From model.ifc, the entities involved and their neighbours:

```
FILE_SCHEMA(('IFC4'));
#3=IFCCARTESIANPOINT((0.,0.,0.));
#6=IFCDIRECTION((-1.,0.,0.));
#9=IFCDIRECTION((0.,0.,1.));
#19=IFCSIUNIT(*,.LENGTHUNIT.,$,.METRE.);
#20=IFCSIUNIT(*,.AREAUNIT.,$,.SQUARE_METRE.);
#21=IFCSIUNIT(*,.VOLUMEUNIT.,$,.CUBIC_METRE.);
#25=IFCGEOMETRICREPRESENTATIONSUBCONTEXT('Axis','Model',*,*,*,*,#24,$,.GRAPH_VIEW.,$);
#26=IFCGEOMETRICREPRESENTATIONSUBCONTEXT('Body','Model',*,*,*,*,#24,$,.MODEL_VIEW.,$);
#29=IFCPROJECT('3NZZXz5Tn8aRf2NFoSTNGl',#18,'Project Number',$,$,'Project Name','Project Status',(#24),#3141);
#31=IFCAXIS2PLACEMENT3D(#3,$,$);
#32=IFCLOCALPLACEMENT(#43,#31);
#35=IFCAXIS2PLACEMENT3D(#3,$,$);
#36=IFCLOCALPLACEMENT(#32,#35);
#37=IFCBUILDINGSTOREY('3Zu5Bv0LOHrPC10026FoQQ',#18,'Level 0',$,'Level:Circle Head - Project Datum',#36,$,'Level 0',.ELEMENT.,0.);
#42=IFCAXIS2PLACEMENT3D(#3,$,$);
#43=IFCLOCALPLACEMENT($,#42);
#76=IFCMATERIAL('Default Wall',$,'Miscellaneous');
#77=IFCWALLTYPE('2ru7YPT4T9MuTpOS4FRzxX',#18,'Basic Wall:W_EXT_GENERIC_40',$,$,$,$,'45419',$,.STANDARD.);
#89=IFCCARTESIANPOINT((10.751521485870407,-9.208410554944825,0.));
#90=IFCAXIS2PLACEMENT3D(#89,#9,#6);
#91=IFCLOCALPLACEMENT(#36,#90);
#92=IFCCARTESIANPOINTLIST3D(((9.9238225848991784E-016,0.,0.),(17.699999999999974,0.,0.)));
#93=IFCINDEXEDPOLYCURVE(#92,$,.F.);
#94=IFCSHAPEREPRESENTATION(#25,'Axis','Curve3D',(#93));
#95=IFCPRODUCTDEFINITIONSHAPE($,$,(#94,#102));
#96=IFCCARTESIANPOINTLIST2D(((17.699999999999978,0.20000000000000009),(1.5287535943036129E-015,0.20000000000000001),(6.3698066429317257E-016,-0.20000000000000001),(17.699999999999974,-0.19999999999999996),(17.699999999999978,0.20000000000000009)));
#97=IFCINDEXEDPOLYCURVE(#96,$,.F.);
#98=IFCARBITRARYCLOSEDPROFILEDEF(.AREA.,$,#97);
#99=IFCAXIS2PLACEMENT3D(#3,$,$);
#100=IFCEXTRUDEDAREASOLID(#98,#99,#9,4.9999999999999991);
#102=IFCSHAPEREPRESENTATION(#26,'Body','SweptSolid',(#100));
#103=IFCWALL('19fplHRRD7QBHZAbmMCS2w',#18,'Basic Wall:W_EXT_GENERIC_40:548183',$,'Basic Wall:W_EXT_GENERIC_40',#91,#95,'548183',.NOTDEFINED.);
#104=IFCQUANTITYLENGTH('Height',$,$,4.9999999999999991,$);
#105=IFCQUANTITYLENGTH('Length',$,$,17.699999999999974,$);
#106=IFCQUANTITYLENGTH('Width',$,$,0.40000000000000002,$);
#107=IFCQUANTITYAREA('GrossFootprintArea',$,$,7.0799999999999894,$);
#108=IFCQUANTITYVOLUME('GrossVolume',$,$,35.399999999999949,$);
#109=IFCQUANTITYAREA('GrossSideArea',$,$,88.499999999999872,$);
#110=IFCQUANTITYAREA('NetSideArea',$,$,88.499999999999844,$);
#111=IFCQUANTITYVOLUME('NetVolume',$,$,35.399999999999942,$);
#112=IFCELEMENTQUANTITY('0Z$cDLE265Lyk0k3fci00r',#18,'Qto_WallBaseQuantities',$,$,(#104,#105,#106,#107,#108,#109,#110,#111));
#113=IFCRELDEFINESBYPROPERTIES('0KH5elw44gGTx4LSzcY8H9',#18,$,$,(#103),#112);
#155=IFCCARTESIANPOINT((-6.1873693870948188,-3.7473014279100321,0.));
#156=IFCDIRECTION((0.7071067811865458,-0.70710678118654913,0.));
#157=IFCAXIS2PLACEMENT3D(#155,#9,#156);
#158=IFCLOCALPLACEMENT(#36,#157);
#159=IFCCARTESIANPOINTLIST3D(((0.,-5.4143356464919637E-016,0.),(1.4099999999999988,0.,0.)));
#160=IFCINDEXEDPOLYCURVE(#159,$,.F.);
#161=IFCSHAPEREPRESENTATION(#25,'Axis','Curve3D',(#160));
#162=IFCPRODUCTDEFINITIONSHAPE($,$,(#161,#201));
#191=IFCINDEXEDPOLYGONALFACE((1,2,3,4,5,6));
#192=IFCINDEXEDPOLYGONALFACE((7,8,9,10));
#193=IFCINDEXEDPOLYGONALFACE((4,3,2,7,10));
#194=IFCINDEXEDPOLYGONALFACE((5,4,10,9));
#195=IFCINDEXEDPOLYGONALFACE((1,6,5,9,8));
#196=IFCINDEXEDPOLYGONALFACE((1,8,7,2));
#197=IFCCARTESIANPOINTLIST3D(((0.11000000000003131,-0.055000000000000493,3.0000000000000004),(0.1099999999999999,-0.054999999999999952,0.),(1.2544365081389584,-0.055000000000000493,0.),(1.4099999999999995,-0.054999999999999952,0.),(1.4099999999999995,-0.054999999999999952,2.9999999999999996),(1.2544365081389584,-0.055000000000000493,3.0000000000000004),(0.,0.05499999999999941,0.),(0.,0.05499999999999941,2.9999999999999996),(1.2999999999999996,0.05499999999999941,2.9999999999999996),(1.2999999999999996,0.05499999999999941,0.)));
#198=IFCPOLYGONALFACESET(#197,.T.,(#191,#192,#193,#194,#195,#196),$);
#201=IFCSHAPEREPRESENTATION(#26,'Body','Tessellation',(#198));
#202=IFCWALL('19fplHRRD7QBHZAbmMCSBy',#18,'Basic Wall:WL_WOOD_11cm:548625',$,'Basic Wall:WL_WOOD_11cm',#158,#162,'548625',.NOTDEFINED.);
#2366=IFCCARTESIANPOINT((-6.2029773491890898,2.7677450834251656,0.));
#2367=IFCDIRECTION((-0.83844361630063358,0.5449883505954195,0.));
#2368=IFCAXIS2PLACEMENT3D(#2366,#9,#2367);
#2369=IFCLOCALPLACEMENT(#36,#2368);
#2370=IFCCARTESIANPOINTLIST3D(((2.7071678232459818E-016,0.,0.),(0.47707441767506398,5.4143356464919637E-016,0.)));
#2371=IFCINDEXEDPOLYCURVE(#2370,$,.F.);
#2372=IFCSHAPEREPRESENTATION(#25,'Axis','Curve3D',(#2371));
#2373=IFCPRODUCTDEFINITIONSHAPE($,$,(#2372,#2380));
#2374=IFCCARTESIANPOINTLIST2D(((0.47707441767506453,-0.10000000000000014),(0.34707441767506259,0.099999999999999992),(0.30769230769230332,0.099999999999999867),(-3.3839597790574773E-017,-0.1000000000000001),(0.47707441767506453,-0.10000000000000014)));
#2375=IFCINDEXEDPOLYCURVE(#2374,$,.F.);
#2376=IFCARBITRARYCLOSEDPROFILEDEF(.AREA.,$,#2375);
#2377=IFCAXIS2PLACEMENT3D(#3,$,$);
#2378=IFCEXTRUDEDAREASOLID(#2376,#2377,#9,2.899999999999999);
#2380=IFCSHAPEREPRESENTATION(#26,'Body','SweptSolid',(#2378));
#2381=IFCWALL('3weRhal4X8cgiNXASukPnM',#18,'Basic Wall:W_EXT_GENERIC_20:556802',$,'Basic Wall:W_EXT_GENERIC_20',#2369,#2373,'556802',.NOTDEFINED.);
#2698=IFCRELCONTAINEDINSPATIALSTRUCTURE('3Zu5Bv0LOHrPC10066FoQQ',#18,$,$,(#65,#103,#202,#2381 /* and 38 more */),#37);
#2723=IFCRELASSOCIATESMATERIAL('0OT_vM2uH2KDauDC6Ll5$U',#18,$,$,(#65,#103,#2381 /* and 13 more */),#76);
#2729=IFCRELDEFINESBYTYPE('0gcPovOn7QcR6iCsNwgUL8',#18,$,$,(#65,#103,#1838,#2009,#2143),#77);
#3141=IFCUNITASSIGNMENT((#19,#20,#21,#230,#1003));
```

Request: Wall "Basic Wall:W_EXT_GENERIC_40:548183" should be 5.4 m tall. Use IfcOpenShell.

```python
import ifcopenshell
import ifcopenshell.api.pset
import ifcopenshell.geom
import ifcopenshell.util.element
import ifcopenshell.util.representation
import ifcopenshell.util.shape
import ifcopenshell.util.unit

model = ifcopenshell.open("model.ifc")
unit_scale = ifcopenshell.util.unit.calculate_unit_scale(model)
area_scale = ifcopenshell.util.unit.calculate_unit_scale(model, "AREAUNIT")
volume_scale = ifcopenshell.util.unit.calculate_unit_scale(model, "VOLUMEUNIT")
settings = ifcopenshell.geom.settings()


def volume(element):
    """Net volume in cubic metres, openings subtracted."""
    shape = ifcopenshell.geom.create_shape(settings, element)
    return ifcopenshell.util.shape.get_volume(shape.geometry)


wall = model.by_guid("19fplHRRD7QBHZAbmMCS2w")
before = volume(wall)

body = ifcopenshell.util.representation.get_representation(wall, "Model", "Body")
solid = body.Items[0]
old_height = solid.Depth
solid.Depth = 5.4
after = volume(wall)
thickness = 0.4  # wall thickness in metres

# Update the stored height, areas and volumes.
qto = model.by_id(ifcopenshell.util.element.get_pset(wall, "Qto_WallBaseQuantities", should_inherit=False)["id"])
ifcopenshell.api.pset.edit_qto(model, qto=qto, properties={
    "Height": solid.Depth,
    "GrossVolume": ifcopenshell.util.element.get_pset(wall, "Qto_WallBaseQuantities", "GrossVolume") * solid.Depth / old_height,
    "GrossSideArea": ifcopenshell.util.element.get_pset(wall, "Qto_WallBaseQuantities", "GrossSideArea") * solid.Depth / old_height,
    "NetSideArea": after / thickness / area_scale,
    "NetVolume": after / volume_scale,
})

print(f"height {old_height:g} -> {solid.Depth:g}, volume {before:.3f} -> {after:.3f} m3")

model.write("model_rev.ifc")
```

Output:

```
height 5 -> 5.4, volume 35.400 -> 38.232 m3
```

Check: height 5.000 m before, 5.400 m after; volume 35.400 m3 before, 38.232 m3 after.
